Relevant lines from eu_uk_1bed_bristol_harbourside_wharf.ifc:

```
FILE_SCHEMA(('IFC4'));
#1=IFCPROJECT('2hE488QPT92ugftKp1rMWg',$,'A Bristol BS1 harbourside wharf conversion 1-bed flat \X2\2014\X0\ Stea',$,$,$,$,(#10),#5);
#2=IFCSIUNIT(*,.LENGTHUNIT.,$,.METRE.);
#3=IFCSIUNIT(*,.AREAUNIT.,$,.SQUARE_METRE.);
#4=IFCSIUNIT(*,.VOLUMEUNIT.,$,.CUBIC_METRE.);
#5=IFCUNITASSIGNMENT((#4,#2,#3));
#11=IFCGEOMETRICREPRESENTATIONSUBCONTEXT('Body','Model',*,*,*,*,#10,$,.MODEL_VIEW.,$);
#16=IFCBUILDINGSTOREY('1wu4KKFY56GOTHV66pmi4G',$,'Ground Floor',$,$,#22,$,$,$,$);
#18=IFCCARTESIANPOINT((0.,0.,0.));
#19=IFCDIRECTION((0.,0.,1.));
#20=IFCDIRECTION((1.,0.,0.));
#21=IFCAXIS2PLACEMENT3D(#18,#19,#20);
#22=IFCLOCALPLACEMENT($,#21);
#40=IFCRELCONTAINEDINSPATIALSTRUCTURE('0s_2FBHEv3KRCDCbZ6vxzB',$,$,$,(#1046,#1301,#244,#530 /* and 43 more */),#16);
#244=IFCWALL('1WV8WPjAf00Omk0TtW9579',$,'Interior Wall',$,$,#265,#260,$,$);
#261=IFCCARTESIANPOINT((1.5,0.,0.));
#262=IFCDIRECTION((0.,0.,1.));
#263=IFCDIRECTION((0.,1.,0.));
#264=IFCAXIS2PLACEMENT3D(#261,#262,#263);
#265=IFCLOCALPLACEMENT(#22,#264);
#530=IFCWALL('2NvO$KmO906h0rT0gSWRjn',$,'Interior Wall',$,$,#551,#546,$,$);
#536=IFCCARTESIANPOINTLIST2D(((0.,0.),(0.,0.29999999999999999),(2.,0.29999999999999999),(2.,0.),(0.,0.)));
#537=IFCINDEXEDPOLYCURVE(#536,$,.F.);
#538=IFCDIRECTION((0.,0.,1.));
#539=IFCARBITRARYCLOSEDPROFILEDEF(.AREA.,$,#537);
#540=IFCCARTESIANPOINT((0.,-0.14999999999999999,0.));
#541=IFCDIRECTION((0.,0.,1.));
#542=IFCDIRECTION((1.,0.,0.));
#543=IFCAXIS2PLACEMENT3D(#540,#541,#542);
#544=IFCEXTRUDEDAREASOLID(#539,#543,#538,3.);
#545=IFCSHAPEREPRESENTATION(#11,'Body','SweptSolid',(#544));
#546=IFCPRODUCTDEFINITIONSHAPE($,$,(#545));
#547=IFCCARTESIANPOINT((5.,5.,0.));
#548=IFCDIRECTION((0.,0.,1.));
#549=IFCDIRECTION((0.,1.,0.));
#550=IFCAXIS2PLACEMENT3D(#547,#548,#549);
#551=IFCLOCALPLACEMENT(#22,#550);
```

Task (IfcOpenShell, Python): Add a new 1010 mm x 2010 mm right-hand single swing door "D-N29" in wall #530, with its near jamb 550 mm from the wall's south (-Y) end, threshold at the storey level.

```python
import numpy as np
import ifcopenshell
import ifcopenshell.api.feature
import ifcopenshell.api.geometry
import ifcopenshell.api.root
import ifcopenshell.api.spatial
import ifcopenshell.geom
import ifcopenshell.util.element
import ifcopenshell.util.placement
import ifcopenshell.util.representation
import ifcopenshell.util.shape
import ifcopenshell.util.unit

model = ifcopenshell.open("eu_uk_1bed_bristol_harbourside_wharf.ifc")
unit_scale = ifcopenshell.util.unit.calculate_unit_scale(model)
settings = ifcopenshell.geom.settings()


def volume(element):
    """Net volume in cubic metres, openings subtracted."""
    shape = ifcopenshell.geom.create_shape(settings, element)
    return ifcopenshell.util.shape.get_volume(shape.geometry)


wall = model.by_id(530)
storey = ifcopenshell.util.element.get_container(wall, ifc_class="IfcBuildingStorey")
context = ifcopenshell.util.representation.get_context(model, "Model", "Body", "MODEL_VIEW")
before = volume(wall)

width, height, from_end, sill = 1.01, 2.01, 0.55, 0.0  # metres

# The wall runs along its own X axis, and the end named is its -X end.
wall_shape = ifcopenshell.geom.create_shape(settings, wall)
x, y, z = ifcopenshell.util.shape.get_vertices(wall_shape.geometry).T
start = x.min() + from_end
face, thickness = float(y.min()), float(y.max() - y.min())
wall_matrix = ifcopenshell.util.placement.get_local_placement(wall.ObjectPlacement)
level = ifcopenshell.util.placement.get_local_placement(storey.ObjectPlacement)[2, 3]


def in_wall(x, y):
    """Placement at x, y metres in the wall's axes, at sill height."""
    matrix = wall_matrix.copy()
    matrix[:, 3] = wall_matrix @ np.array([x / unit_scale, y / unit_scale, 0.0, 1.0])
    matrix[2, 3] = level + sill / unit_scale
    return matrix


# Opening: a box that overshoots both wall faces by 50 mm.
opening = ifcopenshell.api.root.create_entity(model, ifc_class="IfcOpeningElement", predefined_type="OPENING")
box = ifcopenshell.api.geometry.add_wall_representation(
    model, context=context, length=width, height=height, thickness=thickness + 0.1
)
ifcopenshell.api.geometry.assign_representation(model, product=opening, representation=box)
ifcopenshell.api.geometry.edit_object_placement(model, product=opening, matrix=in_wall(start, face - 0.05), is_si=False)
ifcopenshell.api.feature.add_feature(model, feature=opening, element=wall)

door = ifcopenshell.api.root.create_entity(model, ifc_class="IfcDoor", name="D-N29", predefined_type="DOOR")
door.OverallWidth, door.OverallHeight = width / unit_scale, height / unit_scale
door.OperationType = "SINGLE_SWING_RIGHT"
body = ifcopenshell.api.geometry.add_door_representation(
    model,
    context=context,
    overall_width=door.OverallWidth,
    overall_height=door.OverallHeight,
    operation_type="SINGLE_SWING_RIGHT",
    lining_properties={"LiningDepth": thickness / unit_scale, "ThresholdDepth": thickness / unit_scale},
)
ifcopenshell.api.geometry.assign_representation(model, product=door, representation=body)
ifcopenshell.api.spatial.assign_container(model, products=[door], relating_structure=storey)
ifcopenshell.api.feature.add_filling(model, opening=opening, element=door)

# The lining spans the wall, so the door starts at the wall face.
ifcopenshell.api.geometry.edit_object_placement(model, product=door, matrix=in_wall(start, face), is_si=False)

after = volume(wall)

print(f"wall volume {before:.3f} -> {after:.3f} m3")

model.write("eu_uk_1bed_bristol_harbourside_wharf_updated.ifc")
```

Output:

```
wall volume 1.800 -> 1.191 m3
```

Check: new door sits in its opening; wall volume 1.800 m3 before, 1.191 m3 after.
